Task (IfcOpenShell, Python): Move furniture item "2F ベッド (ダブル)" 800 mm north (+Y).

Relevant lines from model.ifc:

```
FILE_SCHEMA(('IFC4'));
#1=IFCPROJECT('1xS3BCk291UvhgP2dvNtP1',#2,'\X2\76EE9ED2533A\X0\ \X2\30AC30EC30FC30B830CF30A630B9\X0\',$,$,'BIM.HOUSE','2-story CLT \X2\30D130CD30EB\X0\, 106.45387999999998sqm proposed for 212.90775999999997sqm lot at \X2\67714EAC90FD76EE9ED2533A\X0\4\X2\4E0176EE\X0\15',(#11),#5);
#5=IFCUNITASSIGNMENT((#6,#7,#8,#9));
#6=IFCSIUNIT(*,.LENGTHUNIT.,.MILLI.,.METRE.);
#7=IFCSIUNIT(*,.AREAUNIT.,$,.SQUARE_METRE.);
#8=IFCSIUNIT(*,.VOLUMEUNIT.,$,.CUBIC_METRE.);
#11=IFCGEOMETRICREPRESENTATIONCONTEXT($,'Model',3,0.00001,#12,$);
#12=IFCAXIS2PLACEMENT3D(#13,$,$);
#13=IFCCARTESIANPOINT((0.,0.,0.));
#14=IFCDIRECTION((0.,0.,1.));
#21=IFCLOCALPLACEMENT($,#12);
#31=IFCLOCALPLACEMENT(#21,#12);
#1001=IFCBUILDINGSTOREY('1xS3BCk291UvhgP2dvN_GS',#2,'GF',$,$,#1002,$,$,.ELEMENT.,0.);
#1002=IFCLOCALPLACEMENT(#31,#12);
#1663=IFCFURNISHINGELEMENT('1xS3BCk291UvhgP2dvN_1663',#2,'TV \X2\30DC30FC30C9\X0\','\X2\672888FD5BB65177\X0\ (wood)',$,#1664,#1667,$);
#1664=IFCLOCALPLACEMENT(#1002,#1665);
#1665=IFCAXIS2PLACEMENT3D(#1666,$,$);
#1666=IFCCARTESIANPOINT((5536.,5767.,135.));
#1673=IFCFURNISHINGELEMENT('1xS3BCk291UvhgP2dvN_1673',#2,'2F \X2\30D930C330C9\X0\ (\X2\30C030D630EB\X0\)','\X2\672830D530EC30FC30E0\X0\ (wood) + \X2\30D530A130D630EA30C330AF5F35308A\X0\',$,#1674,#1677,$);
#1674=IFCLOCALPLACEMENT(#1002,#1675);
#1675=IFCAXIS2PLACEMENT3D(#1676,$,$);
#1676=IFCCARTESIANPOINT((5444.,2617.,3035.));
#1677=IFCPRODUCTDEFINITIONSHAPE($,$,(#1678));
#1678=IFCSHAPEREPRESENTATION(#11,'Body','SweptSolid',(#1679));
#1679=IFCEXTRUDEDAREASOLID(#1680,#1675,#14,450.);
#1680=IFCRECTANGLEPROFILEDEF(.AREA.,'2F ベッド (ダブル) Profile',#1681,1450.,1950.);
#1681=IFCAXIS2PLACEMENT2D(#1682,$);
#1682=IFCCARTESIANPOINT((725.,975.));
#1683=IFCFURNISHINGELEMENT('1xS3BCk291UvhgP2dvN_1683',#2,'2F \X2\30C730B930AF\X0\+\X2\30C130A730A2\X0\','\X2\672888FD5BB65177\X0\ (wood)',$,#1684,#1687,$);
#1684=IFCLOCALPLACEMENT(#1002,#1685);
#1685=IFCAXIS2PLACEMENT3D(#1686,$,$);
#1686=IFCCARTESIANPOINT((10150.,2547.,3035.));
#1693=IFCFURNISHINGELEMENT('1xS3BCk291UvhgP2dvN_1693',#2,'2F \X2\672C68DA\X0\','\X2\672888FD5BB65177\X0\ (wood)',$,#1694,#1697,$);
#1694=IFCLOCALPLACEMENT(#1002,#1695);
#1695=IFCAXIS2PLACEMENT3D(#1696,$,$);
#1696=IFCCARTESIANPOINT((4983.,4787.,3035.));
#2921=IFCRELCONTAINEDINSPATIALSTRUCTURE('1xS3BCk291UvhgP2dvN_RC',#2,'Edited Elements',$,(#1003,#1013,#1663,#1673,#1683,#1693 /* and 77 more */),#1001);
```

```python
import ifcopenshell
import ifcopenshell.api.geometry
import ifcopenshell.util.placement
import ifcopenshell.util.unit

model = ifcopenshell.open("model.ifc")
unit_scale = ifcopenshell.util.unit.calculate_unit_scale(model)

item = model.by_guid("1xS3BCk291UvhgP2dvN_1673")
matrix = ifcopenshell.util.placement.get_local_placement(item.ObjectPlacement)
matrix[1, 3] += 0.8 / unit_scale
ifcopenshell.api.geometry.edit_object_placement(model, product=item, matrix=matrix, is_si=False)

print(ifcopenshell.util.placement.get_local_placement(item.ObjectPlacement).round(3) + 0.0)

model.write("model-out.ifc")
```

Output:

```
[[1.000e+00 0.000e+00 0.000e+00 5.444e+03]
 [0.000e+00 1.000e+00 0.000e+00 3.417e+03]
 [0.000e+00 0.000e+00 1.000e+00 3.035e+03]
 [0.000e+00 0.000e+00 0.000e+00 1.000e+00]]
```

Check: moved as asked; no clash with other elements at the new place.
